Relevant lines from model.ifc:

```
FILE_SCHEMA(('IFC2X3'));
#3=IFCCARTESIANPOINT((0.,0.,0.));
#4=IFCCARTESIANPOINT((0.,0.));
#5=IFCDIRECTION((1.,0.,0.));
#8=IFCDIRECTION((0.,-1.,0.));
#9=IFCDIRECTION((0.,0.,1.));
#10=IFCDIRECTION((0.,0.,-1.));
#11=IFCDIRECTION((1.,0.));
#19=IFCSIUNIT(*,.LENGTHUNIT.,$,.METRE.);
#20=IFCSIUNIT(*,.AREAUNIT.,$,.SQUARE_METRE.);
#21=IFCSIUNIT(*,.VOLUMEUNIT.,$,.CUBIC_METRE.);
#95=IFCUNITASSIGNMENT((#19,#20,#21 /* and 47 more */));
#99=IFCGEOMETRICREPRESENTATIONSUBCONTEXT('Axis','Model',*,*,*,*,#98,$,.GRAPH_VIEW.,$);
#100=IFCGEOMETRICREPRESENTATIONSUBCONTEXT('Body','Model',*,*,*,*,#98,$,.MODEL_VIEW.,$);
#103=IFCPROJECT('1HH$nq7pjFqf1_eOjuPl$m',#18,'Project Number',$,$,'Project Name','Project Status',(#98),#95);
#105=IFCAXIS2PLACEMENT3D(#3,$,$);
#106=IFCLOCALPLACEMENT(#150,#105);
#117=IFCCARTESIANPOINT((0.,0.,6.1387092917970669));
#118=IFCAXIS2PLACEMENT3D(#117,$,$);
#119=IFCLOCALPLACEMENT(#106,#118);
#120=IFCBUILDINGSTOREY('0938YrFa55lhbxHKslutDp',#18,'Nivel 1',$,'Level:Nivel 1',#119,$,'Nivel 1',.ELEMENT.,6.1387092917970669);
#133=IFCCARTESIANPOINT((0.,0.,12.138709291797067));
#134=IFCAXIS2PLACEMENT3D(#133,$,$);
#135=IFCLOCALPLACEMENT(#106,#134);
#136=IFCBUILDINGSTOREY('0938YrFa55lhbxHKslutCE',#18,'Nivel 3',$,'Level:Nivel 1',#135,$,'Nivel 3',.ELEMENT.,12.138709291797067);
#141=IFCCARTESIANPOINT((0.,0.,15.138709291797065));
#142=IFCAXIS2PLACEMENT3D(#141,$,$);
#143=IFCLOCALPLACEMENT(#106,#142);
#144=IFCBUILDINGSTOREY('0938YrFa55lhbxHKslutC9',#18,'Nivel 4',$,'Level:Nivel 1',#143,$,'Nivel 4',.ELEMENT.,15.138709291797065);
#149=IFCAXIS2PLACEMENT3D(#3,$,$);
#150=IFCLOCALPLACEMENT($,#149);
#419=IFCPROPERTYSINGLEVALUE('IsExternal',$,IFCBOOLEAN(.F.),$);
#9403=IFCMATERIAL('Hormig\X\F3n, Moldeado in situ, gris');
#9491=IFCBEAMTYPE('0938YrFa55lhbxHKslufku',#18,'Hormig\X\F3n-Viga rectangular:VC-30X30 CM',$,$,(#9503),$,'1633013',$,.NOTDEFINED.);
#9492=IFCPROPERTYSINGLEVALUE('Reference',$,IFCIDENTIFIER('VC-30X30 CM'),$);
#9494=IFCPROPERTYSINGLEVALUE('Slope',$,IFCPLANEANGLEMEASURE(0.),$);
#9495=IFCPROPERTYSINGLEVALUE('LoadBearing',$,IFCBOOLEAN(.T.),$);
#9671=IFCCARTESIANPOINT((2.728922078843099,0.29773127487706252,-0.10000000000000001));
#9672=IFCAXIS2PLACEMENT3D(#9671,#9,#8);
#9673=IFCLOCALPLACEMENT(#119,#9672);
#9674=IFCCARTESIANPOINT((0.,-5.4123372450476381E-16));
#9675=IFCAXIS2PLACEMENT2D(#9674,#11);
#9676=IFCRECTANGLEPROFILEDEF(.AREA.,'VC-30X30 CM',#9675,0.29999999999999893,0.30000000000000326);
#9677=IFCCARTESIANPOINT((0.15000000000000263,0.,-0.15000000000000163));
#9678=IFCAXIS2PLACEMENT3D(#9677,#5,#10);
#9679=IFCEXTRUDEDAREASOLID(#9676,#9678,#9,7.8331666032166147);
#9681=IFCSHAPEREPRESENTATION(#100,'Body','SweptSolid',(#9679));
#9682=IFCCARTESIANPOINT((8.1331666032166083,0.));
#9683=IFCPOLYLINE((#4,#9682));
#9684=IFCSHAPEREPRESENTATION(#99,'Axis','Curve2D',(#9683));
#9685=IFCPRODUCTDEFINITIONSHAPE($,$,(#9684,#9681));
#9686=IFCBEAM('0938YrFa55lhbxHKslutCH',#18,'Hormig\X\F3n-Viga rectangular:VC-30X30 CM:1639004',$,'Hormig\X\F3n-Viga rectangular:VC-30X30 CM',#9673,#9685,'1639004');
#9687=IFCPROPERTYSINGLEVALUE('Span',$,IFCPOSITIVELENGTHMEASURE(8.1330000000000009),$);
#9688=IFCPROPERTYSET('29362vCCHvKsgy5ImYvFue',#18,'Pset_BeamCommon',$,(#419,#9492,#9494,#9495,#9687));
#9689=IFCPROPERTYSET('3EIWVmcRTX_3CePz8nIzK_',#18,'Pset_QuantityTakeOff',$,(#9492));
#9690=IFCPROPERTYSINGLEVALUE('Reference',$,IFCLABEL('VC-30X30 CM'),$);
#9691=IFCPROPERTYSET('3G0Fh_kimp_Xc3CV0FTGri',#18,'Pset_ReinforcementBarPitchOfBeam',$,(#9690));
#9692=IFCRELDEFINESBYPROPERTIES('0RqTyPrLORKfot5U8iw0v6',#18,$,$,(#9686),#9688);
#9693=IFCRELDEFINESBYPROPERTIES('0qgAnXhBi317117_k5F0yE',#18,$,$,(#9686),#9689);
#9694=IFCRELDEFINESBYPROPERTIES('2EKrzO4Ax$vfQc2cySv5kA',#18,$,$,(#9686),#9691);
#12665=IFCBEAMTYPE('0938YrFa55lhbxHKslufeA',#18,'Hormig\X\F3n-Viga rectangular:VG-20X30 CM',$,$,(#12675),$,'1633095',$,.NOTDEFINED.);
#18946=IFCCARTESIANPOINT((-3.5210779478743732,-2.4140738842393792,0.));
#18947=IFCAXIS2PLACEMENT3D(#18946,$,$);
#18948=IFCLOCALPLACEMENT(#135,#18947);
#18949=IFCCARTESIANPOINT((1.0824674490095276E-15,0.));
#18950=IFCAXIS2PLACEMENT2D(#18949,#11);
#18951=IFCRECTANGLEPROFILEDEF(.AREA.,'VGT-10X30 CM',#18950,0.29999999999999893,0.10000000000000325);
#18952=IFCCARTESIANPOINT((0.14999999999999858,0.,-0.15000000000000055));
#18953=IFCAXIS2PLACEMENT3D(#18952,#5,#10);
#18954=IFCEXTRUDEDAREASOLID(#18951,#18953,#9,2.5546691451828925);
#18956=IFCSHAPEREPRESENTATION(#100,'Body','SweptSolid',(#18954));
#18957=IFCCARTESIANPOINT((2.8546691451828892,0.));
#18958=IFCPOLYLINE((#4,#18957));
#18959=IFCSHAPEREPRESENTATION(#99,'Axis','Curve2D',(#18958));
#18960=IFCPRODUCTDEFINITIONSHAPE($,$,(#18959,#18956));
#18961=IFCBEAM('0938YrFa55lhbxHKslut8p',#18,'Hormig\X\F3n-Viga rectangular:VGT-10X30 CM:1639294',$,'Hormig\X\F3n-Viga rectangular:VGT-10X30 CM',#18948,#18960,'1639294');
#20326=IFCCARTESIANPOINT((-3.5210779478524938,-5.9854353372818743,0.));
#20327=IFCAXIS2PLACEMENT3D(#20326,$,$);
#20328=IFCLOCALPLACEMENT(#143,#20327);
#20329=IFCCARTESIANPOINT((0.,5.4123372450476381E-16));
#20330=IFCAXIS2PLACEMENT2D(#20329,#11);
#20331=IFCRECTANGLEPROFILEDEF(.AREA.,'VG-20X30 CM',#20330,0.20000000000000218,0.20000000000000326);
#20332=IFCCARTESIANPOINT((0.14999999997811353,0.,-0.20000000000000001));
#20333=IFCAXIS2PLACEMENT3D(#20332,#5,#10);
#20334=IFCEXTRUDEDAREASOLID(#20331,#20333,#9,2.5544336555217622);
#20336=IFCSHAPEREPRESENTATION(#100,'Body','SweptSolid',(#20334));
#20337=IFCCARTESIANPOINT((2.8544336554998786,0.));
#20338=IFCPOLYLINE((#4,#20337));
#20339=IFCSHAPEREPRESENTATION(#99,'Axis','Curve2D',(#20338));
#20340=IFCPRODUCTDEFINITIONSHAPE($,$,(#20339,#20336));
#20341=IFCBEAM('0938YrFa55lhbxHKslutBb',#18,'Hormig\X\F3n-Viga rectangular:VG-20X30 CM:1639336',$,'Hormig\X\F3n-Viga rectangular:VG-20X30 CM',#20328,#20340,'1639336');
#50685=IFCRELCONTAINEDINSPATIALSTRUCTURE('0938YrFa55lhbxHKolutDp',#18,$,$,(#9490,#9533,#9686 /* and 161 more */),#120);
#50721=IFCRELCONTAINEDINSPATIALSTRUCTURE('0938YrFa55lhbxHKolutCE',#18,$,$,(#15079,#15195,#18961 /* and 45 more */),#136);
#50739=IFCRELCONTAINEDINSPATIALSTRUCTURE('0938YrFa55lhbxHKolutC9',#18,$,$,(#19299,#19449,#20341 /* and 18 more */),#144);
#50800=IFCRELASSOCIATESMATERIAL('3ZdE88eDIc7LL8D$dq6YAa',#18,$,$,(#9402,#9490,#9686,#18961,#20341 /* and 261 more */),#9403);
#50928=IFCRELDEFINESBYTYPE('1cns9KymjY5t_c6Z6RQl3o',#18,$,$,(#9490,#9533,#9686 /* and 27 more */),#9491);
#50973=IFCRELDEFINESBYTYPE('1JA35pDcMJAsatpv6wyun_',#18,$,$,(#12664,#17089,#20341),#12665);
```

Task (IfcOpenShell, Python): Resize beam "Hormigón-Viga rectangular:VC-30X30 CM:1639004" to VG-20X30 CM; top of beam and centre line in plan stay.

```python
import ifcopenshell
import ifcopenshell.api.pset
import ifcopenshell.api.type
import ifcopenshell.util.element
import ifcopenshell.util.representation

model = ifcopenshell.open("model.ifc")

member = model.by_id(9686)
source = next(p for p in model.by_type("IfcRectangleProfileDef") if p.ProfileName == "VG-20X30 CM")

body = ifcopenshell.util.representation.get_representation(member, "Model", "Body")
solid = body.Items[0]
old_profile = solid.SweptArea

# Copy the section's sizes but keep this member's own profile position.
profile = ifcopenshell.util.element.copy(model, source)
# Profiles are centred, so shift by half the change in depth to hold the top.
shift = (old_profile.XDim - profile.XDim) / 2
x, y = old_profile.Position.Location.Coordinates
up = (-1.0, 0.0)  # upwards, in the solid's own plane
location = model.createIfcCartesianPoint((x + up[0] * shift, y + up[1] * shift))
profile.Position = model.createIfcAxis2Placement2D(location, old_profile.Position.RefDirection)
solid.SweptArea = profile
if not model.get_total_inverses(old_profile):
    ifcopenshell.util.element.remove_deep2(model, old_profile)

new_type = model.by_id(12665)
ifcopenshell.api.type.assign_type(
    model, related_objects=[member], relating_type=new_type, should_map_representations=False
)
member.Name = member.Name.replace("VC-30X30 CM", "VG-20X30 CM")
member.ObjectType = "Hormigón-Viga rectangular:VG-20X30 CM"
pset = model.by_id(ifcopenshell.util.element.get_pset(member, "Pset_BeamCommon", should_inherit=False)["id"])
ifcopenshell.api.pset.edit_pset(model, pset=pset, properties={"Reference": "VG-20X30 CM"})
pset = model.by_id(ifcopenshell.util.element.get_pset(member, "Pset_QuantityTakeOff", should_inherit=False)["id"])
ifcopenshell.api.pset.edit_pset(model, pset=pset, properties={"Reference": "VG-20X30 CM"})
pset = model.by_id(ifcopenshell.util.element.get_pset(member, "Pset_ReinforcementBarPitchOfBeam", should_inherit=False)["id"])
ifcopenshell.api.pset.edit_pset(model, pset=pset, properties={"Reference": "VG-20X30 CM"})

print(solid.SweptArea)

model.write("model-out.ifc")
```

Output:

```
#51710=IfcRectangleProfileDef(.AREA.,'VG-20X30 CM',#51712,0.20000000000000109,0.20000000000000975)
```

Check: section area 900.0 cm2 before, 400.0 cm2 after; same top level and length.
